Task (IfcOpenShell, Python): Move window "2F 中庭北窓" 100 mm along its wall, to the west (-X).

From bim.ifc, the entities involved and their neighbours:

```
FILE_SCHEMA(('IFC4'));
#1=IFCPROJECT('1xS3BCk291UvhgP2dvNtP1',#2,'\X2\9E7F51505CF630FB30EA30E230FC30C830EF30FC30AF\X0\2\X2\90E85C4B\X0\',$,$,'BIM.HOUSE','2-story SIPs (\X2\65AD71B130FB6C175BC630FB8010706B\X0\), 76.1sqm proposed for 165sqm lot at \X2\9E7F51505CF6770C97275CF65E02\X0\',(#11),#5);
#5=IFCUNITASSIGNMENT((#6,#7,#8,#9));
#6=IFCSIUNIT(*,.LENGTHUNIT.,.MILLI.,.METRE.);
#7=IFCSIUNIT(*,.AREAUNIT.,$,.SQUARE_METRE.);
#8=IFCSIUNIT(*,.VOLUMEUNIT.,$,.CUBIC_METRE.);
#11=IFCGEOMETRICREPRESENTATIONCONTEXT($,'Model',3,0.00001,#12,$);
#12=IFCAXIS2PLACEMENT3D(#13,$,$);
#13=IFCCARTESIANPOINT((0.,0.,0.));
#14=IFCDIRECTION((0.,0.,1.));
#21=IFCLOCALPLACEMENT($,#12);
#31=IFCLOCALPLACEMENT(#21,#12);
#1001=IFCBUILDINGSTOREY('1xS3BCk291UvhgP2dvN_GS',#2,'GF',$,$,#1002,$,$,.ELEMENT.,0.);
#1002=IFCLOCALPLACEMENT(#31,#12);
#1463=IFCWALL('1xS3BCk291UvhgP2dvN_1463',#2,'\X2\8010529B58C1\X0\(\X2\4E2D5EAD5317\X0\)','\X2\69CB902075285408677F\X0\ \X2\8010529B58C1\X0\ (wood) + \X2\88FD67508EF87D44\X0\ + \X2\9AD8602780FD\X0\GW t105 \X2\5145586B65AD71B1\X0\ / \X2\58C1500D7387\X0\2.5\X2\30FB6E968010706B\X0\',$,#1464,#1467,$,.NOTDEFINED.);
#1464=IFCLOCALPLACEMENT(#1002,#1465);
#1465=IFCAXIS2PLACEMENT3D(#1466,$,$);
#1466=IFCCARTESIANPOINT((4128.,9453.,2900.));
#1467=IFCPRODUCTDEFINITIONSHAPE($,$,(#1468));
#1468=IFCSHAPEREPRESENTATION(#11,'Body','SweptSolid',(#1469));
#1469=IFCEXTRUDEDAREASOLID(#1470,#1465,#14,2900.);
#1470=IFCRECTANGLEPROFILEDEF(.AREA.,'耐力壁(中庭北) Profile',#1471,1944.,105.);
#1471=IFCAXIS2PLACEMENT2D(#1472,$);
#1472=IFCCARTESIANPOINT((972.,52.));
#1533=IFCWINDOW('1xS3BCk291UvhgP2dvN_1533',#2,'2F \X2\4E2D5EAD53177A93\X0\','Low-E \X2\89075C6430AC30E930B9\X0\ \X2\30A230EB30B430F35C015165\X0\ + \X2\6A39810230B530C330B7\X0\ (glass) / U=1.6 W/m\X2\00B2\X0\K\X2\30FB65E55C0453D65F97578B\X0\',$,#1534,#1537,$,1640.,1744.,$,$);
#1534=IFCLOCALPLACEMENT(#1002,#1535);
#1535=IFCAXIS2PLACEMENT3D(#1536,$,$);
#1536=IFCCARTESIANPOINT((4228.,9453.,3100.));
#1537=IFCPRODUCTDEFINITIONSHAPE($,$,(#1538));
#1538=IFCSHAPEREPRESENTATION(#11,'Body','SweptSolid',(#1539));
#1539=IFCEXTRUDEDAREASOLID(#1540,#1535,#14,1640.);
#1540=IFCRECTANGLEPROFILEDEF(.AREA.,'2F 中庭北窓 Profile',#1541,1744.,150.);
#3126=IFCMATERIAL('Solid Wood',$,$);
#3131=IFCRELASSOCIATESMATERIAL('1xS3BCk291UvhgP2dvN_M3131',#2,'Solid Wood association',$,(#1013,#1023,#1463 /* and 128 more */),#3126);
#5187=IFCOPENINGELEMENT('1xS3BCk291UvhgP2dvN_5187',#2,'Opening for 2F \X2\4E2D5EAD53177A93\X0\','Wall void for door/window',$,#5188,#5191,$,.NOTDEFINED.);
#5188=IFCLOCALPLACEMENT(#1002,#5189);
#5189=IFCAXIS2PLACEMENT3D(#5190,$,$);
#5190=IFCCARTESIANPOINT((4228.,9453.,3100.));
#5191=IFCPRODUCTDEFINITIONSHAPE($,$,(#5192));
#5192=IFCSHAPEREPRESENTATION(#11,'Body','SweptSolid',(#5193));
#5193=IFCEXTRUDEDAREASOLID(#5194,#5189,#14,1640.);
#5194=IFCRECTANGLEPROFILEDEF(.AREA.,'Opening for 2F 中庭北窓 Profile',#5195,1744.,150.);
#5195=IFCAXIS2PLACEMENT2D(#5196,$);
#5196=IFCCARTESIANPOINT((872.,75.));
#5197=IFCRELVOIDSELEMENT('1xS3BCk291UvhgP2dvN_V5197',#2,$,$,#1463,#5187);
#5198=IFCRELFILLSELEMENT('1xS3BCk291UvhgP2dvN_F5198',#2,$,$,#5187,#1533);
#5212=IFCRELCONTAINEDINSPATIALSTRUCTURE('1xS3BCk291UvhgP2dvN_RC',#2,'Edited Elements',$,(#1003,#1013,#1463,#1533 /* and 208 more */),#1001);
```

```python
import ifcopenshell
import ifcopenshell.api.geometry
import ifcopenshell.util.placement
import ifcopenshell.util.unit

model = ifcopenshell.open("bim.ifc")
unit_scale = ifcopenshell.util.unit.calculate_unit_scale(model)

window = model.by_id(1533)
opening = window.FillsVoids[0].RelatingOpeningElement
wall = opening.VoidsElements[0].RelatingBuildingElement

wall_matrix = ifcopenshell.util.placement.get_local_placement(wall.ObjectPlacement)
shift = wall_matrix[:3, 0] * -0.1 / unit_scale
before = ifcopenshell.util.placement.get_local_placement(window.ObjectPlacement)[:3, 3].copy()

# The window is not placed relative to its opening, so move both.
for product in (opening, window):
    matrix = ifcopenshell.util.placement.get_local_placement(product.ObjectPlacement)
    matrix[:3, 3] += shift
    ifcopenshell.api.geometry.edit_object_placement(model, product=product, matrix=matrix, is_si=False)

after = ifcopenshell.util.placement.get_local_placement(window.ObjectPlacement)[:3, 3]
print("window moved by", (after - before).round(3) + 0.0)

model.write("bim_v2.ifc")
```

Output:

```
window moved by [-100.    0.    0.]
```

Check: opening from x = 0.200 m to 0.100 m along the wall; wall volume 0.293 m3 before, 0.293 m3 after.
